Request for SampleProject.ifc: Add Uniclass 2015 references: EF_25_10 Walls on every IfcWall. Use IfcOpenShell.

First a look at what the model holds.

```python
import ifcopenshell

model = ifcopenshell.open("SampleProject.ifc")
print(model.schema)
print("classifications:", [c.Name for c in model.by_type("IfcClassification")])
for ifc_class in ("IfcDoor", "IfcRoof", "IfcStair", "IfcWall", "IfcWindow"):
    print(ifc_class, len(model.by_type(ifc_class)))
```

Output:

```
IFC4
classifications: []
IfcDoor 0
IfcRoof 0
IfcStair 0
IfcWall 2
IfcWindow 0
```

```python
import ifcopenshell
import ifcopenshell.api.classification

model = ifcopenshell.open("SampleProject.ifc")

system = ifcopenshell.api.classification.add_classification(model, classification="Uniclass 2015")

codes = {
    "IfcWall": ("EF_25_10", "Walls"),
}
for ifc_class, (code, name) in codes.items():
    products = model.by_type(ifc_class)
    ifcopenshell.api.classification.add_reference(
        model, products=products, classification=system, identification=code, name=name
    )
    print(code, len(products))

model.write("SampleProject-out.ifc")
```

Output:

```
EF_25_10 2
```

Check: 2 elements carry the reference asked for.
